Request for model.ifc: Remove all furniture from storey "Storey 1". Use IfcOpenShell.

First a look at what the model holds.

```python
import ifcopenshell
import ifcopenshell.util.element

model = ifcopenshell.open("model.ifc")
print(model.schema)
storey = next(s for s in model.by_type("IfcBuildingStorey") if s.Name == "Storey 1")
furniture = [e for e in ifcopenshell.util.element.get_decomposition(storey) if e.is_a("IfcFurnishingElement")]
seen = {}
for e in furniture:
    element_type = ifcopenshell.util.element.get_type(e)
    name = element_type.Name if element_type not in (None, e) else None
    seen[name] = seen.get(name, 0) + 1
for name, count in sorted(seen.items(), key=str):
    print(count, "x", name)
```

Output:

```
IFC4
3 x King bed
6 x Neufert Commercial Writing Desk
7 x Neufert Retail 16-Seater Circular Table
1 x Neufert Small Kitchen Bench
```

```python
import ifcopenshell
import ifcopenshell.api.root
import ifcopenshell.util.element

model = ifcopenshell.open("model.ifc")

storey = next(s for s in model.by_type("IfcBuildingStorey") if s.Name == "Storey 1")
furniture = [e for e in ifcopenshell.util.element.get_decomposition(storey) if e.is_a("IfcFurnishingElement")]

for e in furniture:
    ifcopenshell.api.root.remove_product(model, product=e)
print(len(furniture), "removed")

model.write("model_v2.ifc")
```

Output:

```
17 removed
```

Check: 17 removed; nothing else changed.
